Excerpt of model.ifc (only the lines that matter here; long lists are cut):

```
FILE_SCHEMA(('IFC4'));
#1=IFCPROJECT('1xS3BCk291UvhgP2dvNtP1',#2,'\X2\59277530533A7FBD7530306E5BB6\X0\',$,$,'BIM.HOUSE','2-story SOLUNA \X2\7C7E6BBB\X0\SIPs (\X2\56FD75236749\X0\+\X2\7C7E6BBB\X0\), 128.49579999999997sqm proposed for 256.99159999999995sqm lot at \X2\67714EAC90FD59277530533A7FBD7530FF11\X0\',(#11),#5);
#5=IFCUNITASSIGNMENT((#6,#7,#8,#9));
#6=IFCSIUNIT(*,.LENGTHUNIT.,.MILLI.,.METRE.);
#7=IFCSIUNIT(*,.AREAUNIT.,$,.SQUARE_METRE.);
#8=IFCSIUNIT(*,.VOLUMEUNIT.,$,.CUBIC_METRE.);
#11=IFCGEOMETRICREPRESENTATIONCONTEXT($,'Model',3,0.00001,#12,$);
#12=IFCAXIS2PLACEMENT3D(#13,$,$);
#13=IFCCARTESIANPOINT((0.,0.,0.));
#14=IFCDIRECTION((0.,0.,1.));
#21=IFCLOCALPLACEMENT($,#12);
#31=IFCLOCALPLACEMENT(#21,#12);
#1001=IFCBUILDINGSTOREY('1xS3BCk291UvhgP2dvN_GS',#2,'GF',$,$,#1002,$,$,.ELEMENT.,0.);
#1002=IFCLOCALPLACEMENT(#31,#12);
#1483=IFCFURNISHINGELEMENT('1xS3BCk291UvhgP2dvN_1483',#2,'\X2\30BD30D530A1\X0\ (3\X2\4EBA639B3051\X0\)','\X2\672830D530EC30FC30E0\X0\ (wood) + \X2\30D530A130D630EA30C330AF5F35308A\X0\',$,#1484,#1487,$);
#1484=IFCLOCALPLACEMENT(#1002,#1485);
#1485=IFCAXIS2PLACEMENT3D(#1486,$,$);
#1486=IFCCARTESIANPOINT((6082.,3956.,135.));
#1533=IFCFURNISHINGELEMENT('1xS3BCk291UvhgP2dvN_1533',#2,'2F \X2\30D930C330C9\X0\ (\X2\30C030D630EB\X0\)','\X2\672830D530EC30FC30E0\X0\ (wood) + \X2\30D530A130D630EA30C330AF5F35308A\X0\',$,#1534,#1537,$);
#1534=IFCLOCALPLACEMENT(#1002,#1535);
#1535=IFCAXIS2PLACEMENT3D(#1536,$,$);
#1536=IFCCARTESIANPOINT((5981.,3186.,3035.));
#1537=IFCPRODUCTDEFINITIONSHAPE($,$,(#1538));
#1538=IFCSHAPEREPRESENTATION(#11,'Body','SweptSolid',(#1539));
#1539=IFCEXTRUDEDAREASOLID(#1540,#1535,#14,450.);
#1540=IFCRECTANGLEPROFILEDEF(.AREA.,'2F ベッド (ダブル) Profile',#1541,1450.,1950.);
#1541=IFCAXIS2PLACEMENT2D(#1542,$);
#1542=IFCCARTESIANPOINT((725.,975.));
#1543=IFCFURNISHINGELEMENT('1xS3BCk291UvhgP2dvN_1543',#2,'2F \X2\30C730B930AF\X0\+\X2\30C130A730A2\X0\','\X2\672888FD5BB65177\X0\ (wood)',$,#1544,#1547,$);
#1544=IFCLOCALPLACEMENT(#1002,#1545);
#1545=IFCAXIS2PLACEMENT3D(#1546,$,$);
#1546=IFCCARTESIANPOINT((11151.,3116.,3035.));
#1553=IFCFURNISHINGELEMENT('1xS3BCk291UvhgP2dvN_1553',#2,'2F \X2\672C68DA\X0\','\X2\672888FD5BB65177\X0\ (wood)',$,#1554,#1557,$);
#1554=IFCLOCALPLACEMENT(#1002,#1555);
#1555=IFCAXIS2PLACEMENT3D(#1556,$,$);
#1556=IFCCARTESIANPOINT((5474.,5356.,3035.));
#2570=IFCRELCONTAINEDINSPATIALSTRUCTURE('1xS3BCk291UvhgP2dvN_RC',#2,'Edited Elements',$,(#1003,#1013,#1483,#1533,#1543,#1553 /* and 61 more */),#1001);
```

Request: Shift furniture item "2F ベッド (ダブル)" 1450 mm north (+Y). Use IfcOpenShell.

```python
import ifcopenshell
import ifcopenshell.api.geometry
import ifcopenshell.util.placement

model = ifcopenshell.open("model.ifc")

item = model.by_guid("1xS3BCk291UvhgP2dvN_1533")
matrix = ifcopenshell.util.placement.get_local_placement(item.ObjectPlacement)
matrix[1, 3] += 1450.0
ifcopenshell.api.geometry.edit_object_placement(model, product=item, matrix=matrix, is_si=False)

print(ifcopenshell.util.placement.get_local_placement(item.ObjectPlacement).round(3) + 0.0)

model.write("model_edited.ifc")
```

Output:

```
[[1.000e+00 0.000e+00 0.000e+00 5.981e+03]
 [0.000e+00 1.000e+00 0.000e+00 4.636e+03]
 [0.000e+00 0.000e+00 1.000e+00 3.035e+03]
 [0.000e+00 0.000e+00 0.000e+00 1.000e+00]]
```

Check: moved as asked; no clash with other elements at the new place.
